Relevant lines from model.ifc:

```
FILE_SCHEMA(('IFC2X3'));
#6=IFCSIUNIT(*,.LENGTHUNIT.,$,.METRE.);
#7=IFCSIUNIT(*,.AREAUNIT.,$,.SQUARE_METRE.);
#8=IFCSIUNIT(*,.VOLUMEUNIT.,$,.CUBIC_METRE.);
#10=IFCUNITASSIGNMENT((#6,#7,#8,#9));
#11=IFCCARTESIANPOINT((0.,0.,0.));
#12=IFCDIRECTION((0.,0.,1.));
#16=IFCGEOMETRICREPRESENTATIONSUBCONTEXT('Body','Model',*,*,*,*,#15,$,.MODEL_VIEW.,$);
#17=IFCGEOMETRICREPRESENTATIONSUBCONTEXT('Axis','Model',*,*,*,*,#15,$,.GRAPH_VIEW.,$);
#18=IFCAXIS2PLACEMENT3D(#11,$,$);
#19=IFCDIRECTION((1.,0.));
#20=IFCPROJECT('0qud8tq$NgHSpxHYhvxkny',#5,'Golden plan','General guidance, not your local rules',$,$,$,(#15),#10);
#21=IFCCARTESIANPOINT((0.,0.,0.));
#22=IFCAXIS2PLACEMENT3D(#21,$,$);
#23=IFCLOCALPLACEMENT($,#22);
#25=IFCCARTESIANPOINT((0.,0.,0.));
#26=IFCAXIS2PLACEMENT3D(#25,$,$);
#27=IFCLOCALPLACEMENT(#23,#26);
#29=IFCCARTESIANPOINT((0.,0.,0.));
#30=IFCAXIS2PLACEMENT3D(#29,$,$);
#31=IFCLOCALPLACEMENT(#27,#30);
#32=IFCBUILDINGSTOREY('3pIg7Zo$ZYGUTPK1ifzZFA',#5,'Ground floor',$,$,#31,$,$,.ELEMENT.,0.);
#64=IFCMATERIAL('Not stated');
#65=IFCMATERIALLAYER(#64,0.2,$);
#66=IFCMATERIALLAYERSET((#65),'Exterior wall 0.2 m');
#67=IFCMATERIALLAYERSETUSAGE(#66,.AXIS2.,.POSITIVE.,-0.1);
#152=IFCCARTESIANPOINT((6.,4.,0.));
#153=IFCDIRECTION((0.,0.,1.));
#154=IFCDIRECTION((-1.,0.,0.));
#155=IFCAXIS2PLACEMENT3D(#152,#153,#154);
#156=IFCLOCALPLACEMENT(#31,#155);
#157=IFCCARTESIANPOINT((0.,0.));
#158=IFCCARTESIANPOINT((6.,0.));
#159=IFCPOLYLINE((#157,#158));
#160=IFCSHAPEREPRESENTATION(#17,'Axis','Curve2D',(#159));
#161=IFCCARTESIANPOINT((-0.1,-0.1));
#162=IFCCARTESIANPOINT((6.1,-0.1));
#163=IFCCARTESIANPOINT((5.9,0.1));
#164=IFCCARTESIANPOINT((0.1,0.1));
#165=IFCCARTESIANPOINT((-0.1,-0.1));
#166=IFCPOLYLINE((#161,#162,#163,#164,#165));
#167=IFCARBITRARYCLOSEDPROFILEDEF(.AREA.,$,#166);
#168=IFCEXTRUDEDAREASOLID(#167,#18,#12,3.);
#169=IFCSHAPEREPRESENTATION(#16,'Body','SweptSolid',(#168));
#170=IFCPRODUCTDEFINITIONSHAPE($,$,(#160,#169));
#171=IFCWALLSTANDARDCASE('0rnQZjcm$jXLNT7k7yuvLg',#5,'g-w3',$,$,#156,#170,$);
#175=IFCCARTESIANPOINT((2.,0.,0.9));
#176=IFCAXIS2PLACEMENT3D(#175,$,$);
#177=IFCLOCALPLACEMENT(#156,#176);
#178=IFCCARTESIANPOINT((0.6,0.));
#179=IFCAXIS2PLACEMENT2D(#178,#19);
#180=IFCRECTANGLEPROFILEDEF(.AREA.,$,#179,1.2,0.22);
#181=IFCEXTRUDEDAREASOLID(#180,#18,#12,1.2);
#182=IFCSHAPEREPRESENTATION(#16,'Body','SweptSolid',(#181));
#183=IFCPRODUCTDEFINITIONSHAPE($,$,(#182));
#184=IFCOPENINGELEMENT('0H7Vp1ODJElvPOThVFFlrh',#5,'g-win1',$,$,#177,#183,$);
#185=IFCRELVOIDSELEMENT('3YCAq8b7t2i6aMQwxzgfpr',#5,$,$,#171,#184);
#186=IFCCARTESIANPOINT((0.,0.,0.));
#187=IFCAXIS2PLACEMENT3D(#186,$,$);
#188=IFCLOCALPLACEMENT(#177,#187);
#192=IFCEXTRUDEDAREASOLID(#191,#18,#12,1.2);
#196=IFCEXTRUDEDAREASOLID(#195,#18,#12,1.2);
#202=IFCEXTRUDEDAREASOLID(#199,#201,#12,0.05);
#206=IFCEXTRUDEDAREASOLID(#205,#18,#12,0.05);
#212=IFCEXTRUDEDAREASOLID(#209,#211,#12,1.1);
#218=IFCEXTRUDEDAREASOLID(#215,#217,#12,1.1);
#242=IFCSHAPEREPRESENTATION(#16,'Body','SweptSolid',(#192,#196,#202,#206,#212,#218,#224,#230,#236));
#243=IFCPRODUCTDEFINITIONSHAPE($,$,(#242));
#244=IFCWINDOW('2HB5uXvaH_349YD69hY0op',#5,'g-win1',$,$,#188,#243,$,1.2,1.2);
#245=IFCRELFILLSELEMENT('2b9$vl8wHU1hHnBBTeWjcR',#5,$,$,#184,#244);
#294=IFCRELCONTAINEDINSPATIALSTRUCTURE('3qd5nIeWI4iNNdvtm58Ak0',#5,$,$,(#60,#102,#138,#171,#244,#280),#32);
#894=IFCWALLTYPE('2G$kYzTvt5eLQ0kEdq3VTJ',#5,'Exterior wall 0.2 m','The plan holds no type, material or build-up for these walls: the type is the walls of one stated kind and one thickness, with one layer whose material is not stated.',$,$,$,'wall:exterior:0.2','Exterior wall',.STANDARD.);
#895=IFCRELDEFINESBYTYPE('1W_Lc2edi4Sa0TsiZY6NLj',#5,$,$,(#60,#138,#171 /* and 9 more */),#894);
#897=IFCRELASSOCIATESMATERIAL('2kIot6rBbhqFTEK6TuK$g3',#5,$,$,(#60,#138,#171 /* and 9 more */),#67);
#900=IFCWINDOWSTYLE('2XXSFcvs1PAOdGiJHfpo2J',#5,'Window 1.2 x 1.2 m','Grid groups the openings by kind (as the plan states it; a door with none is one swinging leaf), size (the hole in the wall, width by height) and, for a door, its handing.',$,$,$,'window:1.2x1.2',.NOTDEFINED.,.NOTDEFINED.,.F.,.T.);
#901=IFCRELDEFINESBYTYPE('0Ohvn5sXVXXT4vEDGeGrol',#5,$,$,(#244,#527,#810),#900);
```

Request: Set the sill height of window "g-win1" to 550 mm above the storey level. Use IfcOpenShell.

```python
import numpy as np
import ifcopenshell
import ifcopenshell.api.geometry
import ifcopenshell.geom
import ifcopenshell.util.element
import ifcopenshell.util.placement
import ifcopenshell.util.shape
import ifcopenshell.util.unit

model = ifcopenshell.open("model.ifc")
unit_scale = ifcopenshell.util.unit.calculate_unit_scale(model)

window = model.by_id(244)
opening = window.FillsVoids[0].RelatingOpeningElement
storey = ifcopenshell.util.element.get_container(window, ifc_class="IfcBuildingStorey")
level = ifcopenshell.util.placement.get_local_placement(storey.ObjectPlacement)[2, 3]

# The opening's origin need not be at the sill, so measure its lowest point.
shape = ifcopenshell.geom.create_shape(ifcopenshell.geom.settings(), opening)
bottom = ifcopenshell.util.shape.get_shape_bottom_elevation(shape, shape.geometry) / unit_scale
dz = level + 0.55 / unit_scale - bottom

shift = np.array([0.0, 0.0, dz])
# The window is placed relative to its opening, so it follows when the opening moves.
matrix = ifcopenshell.util.placement.get_local_placement(opening.ObjectPlacement)
matrix[:3, 3] += shift
ifcopenshell.api.geometry.edit_object_placement(
    model, product=opening, matrix=matrix, is_si=False, should_transform_children=True
)

print(f"moved by {dz * unit_scale:+.3f} m")

model.write("model_rev.ifc")
```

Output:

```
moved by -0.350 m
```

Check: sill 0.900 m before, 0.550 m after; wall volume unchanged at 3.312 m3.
